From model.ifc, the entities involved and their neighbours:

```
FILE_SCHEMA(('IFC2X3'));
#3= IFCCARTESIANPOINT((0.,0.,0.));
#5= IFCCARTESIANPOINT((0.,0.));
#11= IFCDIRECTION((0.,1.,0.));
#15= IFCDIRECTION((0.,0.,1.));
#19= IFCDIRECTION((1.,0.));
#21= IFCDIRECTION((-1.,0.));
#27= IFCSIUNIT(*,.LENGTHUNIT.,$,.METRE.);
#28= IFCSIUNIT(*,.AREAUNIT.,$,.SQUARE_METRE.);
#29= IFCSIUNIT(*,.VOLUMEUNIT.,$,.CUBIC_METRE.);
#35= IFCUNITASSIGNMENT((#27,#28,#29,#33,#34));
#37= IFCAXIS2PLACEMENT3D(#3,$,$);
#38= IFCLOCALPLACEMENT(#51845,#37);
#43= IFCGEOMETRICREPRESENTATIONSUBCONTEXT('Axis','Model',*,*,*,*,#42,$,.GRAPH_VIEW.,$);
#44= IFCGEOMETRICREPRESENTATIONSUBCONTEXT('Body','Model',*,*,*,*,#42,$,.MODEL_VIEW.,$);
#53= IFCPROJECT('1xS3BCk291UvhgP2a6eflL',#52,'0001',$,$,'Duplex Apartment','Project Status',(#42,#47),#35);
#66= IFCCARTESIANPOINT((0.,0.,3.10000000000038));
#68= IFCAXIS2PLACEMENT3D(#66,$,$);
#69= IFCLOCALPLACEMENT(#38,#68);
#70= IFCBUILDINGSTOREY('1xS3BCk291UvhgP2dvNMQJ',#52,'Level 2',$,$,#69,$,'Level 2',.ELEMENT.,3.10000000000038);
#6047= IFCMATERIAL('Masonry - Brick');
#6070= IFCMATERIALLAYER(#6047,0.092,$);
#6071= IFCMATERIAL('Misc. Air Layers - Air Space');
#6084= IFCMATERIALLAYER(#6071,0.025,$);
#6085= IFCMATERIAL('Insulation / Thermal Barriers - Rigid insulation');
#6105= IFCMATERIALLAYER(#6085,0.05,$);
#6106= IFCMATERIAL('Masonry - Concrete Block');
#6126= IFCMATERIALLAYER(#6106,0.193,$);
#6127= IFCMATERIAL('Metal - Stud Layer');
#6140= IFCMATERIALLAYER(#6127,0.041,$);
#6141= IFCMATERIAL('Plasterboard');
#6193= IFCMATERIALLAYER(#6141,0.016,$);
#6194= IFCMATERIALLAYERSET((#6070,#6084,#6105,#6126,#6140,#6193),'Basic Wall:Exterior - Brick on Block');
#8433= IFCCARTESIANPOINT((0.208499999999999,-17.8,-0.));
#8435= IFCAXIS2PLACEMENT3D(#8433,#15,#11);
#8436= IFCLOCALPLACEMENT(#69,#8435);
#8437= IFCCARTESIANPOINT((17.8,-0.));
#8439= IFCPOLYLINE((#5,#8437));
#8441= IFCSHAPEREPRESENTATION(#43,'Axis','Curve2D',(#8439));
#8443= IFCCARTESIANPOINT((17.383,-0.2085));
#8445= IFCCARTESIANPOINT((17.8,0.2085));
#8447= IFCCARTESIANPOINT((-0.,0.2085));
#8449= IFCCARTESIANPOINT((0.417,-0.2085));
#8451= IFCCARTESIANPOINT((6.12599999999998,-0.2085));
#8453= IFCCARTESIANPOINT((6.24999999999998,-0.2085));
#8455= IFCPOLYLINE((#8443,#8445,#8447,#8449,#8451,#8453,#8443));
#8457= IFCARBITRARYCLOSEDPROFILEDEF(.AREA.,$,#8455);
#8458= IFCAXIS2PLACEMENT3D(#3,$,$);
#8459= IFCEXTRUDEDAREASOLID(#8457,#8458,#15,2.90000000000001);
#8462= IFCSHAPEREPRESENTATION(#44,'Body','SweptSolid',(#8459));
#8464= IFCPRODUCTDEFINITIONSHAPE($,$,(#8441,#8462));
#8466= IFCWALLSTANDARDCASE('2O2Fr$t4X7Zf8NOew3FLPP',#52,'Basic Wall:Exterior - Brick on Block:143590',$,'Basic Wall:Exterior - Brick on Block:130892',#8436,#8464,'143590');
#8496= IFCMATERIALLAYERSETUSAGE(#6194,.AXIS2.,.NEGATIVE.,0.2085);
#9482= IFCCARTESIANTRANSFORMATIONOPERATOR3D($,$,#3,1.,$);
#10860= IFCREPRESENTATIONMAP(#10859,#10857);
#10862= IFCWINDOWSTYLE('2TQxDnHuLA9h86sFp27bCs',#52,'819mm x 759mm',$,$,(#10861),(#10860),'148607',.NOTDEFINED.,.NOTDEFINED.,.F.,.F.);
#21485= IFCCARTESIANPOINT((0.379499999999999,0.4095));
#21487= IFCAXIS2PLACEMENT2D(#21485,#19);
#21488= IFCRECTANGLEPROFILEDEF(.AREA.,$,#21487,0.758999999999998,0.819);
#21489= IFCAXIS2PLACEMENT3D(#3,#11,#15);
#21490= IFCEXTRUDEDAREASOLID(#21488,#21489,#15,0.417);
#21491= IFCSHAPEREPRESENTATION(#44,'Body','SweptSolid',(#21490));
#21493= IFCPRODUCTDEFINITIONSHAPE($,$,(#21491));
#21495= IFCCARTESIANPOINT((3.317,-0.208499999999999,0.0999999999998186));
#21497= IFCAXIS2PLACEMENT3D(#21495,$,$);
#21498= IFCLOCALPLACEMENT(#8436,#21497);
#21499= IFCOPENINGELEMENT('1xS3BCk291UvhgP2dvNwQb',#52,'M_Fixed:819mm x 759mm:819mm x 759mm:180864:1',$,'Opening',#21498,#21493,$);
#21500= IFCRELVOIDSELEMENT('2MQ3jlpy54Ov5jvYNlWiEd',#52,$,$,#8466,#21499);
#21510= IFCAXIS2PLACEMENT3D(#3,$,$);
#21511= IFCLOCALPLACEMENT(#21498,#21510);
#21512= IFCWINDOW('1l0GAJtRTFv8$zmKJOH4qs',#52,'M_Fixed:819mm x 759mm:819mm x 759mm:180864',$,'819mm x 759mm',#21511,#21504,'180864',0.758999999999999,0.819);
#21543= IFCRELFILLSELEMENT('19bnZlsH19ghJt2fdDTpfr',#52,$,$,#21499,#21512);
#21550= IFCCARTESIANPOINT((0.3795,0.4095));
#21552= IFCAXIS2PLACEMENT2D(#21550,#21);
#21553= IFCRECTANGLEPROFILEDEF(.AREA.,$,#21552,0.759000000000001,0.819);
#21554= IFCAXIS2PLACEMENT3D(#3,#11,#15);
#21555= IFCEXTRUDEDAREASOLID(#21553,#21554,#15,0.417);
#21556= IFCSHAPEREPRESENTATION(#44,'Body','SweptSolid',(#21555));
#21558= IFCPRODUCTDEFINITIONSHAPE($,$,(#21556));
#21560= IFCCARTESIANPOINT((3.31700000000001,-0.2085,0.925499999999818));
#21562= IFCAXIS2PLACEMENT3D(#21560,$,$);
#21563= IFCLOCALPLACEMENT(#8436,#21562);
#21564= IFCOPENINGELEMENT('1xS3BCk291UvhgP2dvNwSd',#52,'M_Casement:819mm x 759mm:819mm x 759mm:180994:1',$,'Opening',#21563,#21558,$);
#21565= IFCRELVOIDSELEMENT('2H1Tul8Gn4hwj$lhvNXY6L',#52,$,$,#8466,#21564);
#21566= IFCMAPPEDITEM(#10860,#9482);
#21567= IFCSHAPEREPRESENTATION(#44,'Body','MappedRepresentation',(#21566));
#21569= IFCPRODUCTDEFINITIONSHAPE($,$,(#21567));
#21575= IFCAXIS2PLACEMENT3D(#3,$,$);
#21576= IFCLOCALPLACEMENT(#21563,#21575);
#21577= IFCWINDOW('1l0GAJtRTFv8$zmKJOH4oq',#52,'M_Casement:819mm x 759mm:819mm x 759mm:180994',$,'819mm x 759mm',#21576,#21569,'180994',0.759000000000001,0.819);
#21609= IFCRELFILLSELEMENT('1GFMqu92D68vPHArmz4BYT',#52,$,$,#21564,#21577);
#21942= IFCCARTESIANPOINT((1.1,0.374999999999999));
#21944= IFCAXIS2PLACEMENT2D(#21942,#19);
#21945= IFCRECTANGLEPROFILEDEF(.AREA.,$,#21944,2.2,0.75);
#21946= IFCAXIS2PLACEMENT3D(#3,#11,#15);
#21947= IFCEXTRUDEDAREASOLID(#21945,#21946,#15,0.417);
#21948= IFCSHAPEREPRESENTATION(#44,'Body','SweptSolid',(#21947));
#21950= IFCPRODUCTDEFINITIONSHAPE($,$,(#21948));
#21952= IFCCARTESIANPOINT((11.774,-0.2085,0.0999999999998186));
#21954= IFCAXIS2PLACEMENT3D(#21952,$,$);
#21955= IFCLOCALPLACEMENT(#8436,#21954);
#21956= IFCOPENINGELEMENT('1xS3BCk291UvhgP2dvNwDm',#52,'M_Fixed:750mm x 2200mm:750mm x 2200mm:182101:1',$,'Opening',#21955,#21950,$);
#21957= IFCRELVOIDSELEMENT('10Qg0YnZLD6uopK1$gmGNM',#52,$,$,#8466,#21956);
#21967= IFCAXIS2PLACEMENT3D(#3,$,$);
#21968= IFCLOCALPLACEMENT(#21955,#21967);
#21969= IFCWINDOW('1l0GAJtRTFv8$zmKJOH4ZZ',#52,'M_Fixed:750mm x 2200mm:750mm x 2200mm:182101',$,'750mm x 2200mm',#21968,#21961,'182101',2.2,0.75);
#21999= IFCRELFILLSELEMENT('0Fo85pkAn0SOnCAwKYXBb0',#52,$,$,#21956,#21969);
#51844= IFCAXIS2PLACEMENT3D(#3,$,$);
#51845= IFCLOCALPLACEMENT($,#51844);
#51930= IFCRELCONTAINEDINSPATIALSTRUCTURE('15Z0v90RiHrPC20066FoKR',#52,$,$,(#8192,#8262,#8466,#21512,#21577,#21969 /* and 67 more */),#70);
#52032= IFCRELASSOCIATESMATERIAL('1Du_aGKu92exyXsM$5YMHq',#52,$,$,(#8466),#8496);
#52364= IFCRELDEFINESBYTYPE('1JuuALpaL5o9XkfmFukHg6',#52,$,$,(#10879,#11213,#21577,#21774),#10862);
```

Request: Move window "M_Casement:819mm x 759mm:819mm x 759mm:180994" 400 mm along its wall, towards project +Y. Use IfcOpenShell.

```python
import ifcopenshell
import ifcopenshell.api.geometry
import ifcopenshell.util.placement
import ifcopenshell.util.unit

model = ifcopenshell.open("model.ifc")
unit_scale = ifcopenshell.util.unit.calculate_unit_scale(model)

window = model.by_guid("1l0GAJtRTFv8$zmKJOH4oq")
opening = window.FillsVoids[0].RelatingOpeningElement
wall = opening.VoidsElements[0].RelatingBuildingElement

wall_matrix = ifcopenshell.util.placement.get_local_placement(wall.ObjectPlacement)
shift = wall_matrix[:3, 0] * 0.4 / unit_scale
before = ifcopenshell.util.placement.get_local_placement(window.ObjectPlacement)[:3, 3].copy()

# The window is placed relative to its opening, so it follows when the opening moves.
matrix = ifcopenshell.util.placement.get_local_placement(opening.ObjectPlacement)
matrix[:3, 3] += shift
ifcopenshell.api.geometry.edit_object_placement(
    model, product=opening, matrix=matrix, is_si=False, should_transform_children=True
)

after = ifcopenshell.util.placement.get_local_placement(window.ObjectPlacement)[:3, 3]
print("window moved by", (after - before).round(3) + 0.0)

model.write("model-out.ifc")
```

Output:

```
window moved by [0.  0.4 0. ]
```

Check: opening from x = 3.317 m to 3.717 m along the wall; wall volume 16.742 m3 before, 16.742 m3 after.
